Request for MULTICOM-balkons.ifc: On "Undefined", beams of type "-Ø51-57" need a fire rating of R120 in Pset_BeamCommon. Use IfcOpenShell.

First a look at what the model holds.

```python
import ifcopenshell
import ifcopenshell.util.element

model = ifcopenshell.open("MULTICOM-balkons.ifc")
print(model.schema)
storey = next(s for s in model.by_type("IfcBuildingStorey") if s.Name == "Undefined")
beams = [e for e in ifcopenshell.util.element.get_decomposition(storey) if e.is_a("IfcBeam")]
seen = {}
for e in beams:
    element_type = ifcopenshell.util.element.get_type(e)
    key = (element_type.Name if element_type != e and element_type else None, ifcopenshell.util.element.get_pset(e, "Pset_BeamCommon", "FireRating"))
    seen[key] = seen.get(key, 0) + 1
for (name, value), count in sorted(seen.items(), key=str):
    print(count, "x", name, "|", value)
```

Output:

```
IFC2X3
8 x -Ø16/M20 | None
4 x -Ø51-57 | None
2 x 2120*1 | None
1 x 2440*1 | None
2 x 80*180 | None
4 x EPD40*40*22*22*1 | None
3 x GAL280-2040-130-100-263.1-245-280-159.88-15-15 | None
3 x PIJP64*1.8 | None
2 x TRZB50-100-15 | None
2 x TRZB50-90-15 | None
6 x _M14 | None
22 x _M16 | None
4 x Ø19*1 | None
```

```python
import ifcopenshell
import ifcopenshell.api.pset
import ifcopenshell.util.element

model = ifcopenshell.open("MULTICOM-balkons.ifc")

storey = next(s for s in model.by_type("IfcBuildingStorey") if s.Name == "Undefined")
beams = [e for e in ifcopenshell.util.element.get_decomposition(storey) if e.is_a("IfcBeam")]

count = 0
for e in beams:
    element_type = ifcopenshell.util.element.get_type(e)
    if element_type in (None, e) or element_type.Name != "-Ø51-57":
        continue
    # add_pset returns the element's existing set when there is one.
    pset = ifcopenshell.api.pset.add_pset(model, product=e, name="Pset_BeamCommon")
    ifcopenshell.api.pset.edit_pset(model, pset=pset, properties={"FireRating": "R120"})
    count += 1

print(count, "beams updated")

model.write("MULTICOM-balkons_updated.ifc")
```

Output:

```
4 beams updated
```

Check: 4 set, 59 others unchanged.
